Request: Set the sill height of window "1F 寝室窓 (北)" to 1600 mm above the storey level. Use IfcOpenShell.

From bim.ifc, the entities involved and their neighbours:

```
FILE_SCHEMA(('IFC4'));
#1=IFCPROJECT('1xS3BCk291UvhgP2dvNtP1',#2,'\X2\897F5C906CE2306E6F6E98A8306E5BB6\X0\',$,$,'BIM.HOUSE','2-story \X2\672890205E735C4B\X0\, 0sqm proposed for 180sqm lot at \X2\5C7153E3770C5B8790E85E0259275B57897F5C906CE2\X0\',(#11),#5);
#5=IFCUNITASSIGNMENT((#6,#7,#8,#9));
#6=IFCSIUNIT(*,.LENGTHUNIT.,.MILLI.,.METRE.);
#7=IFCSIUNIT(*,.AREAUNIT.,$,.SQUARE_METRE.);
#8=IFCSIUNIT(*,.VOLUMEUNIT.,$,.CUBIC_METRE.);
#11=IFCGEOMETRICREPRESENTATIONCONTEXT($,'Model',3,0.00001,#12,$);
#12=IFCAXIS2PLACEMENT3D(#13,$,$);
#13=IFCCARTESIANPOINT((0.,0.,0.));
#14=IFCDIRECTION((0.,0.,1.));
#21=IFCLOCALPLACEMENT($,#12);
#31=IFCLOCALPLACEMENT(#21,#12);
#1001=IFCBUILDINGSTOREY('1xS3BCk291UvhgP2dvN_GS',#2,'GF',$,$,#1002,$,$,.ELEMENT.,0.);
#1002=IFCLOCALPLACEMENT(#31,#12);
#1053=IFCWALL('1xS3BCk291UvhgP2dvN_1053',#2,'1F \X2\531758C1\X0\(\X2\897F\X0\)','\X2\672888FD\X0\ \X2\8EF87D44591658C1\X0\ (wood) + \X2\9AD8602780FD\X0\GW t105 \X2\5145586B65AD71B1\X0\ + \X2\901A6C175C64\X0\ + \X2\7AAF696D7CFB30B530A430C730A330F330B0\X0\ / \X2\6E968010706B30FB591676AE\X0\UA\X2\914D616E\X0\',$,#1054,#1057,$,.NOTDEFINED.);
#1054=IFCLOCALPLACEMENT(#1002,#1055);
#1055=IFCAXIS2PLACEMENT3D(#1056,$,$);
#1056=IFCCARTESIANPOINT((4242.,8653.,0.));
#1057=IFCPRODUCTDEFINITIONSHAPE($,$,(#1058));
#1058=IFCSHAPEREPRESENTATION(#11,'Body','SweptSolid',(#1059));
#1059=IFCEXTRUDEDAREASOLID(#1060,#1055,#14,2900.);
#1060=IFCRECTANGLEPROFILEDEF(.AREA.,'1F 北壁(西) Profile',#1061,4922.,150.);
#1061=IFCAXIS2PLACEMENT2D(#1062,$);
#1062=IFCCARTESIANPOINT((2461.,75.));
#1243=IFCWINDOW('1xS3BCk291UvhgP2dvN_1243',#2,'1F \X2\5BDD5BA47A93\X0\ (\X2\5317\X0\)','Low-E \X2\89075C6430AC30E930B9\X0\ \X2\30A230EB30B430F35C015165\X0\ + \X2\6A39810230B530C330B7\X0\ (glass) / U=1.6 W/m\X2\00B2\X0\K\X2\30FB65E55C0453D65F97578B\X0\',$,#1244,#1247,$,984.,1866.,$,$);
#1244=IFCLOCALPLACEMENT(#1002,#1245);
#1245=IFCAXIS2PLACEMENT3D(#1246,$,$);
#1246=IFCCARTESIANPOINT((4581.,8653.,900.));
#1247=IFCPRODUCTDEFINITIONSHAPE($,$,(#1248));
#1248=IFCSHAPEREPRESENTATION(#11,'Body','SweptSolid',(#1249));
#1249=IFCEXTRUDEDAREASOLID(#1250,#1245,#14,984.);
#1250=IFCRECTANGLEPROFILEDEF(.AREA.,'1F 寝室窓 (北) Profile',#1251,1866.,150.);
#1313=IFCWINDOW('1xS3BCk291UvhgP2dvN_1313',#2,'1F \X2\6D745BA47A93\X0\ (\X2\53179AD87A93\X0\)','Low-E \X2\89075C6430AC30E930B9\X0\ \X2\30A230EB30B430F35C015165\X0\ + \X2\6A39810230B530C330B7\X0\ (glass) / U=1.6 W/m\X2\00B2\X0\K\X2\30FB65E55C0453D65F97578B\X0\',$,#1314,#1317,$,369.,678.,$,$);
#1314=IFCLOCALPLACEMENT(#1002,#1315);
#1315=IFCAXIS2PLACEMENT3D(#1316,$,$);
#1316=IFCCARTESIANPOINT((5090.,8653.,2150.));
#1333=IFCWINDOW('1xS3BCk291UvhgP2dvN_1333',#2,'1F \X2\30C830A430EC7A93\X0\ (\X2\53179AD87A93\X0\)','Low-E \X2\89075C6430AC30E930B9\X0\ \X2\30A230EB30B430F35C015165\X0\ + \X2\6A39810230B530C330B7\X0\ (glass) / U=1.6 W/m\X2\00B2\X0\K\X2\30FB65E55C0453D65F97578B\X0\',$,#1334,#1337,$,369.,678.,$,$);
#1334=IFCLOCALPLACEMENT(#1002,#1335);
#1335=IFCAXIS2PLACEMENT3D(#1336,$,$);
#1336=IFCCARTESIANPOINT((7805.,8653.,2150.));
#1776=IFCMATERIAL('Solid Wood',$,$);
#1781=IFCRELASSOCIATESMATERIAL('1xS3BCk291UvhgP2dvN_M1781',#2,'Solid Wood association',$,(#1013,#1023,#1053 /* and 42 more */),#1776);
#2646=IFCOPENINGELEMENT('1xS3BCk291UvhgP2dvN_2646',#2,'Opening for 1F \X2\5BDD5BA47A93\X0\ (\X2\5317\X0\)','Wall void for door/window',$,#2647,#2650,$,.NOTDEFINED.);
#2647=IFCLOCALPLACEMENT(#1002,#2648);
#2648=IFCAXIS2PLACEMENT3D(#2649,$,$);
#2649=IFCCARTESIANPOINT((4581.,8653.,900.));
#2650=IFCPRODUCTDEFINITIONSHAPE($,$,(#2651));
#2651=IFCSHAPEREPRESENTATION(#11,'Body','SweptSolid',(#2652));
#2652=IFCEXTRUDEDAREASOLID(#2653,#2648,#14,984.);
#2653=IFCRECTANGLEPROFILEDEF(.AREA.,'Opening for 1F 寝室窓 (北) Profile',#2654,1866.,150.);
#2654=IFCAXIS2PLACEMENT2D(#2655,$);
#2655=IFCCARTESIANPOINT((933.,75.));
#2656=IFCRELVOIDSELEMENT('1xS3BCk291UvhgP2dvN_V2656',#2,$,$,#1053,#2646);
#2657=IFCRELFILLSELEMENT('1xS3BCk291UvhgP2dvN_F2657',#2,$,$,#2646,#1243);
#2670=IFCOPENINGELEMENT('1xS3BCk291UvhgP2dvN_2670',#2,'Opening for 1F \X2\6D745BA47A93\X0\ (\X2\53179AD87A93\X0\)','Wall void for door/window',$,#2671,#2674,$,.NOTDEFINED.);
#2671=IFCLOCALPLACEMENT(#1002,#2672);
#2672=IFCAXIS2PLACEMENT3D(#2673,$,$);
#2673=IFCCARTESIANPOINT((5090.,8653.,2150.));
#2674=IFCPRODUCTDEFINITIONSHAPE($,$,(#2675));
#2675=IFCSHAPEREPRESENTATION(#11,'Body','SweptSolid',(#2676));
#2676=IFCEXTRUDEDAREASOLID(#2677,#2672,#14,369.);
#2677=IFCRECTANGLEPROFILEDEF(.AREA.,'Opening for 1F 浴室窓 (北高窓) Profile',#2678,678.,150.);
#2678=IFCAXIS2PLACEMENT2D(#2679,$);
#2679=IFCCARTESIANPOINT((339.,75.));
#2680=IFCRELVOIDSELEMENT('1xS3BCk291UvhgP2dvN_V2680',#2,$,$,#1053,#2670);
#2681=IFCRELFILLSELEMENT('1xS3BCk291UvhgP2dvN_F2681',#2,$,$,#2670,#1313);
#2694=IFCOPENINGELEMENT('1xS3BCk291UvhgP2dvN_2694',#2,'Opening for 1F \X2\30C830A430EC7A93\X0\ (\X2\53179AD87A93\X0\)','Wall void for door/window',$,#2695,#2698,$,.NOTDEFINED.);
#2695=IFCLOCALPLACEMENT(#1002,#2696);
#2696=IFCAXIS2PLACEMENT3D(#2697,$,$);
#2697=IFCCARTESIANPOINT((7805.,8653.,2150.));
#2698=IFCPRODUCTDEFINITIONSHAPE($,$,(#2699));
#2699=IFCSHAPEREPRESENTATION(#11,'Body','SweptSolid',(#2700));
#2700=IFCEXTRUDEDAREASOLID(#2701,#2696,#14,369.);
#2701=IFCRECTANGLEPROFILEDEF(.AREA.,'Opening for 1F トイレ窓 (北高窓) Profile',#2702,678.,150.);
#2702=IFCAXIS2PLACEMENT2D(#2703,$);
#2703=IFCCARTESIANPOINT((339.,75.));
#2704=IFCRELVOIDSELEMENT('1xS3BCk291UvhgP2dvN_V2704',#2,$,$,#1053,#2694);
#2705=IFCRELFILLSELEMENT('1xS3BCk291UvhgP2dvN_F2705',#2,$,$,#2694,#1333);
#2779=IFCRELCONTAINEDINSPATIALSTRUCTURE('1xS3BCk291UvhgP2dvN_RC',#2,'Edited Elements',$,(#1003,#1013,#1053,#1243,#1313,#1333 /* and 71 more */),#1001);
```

```python
import numpy as np
import ifcopenshell
import ifcopenshell.api.geometry
import ifcopenshell.geom
import ifcopenshell.util.element
import ifcopenshell.util.placement
import ifcopenshell.util.shape
import ifcopenshell.util.unit

model = ifcopenshell.open("bim.ifc")
unit_scale = ifcopenshell.util.unit.calculate_unit_scale(model)

window = model.by_guid("1xS3BCk291UvhgP2dvN_1243")
opening = window.FillsVoids[0].RelatingOpeningElement
storey = ifcopenshell.util.element.get_container(window, ifc_class="IfcBuildingStorey")
level = ifcopenshell.util.placement.get_local_placement(storey.ObjectPlacement)[2, 3]

# The opening's origin need not be at the sill, so measure its lowest point.
shape = ifcopenshell.geom.create_shape(ifcopenshell.geom.settings(), opening)
bottom = ifcopenshell.util.shape.get_shape_bottom_elevation(shape, shape.geometry) / unit_scale
dz = level + 1600.0 - bottom

shift = np.array([0.0, 0.0, dz])
# The window is not placed relative to its opening, so move both.
for product in (opening, window):
    matrix = ifcopenshell.util.placement.get_local_placement(product.ObjectPlacement)
    matrix[:3, 3] += shift
    ifcopenshell.api.geometry.edit_object_placement(model, product=product, matrix=matrix, is_si=False)

print(f"moved by {dz * unit_scale:+.3f} m")

model.write("bim_v2.ifc")
```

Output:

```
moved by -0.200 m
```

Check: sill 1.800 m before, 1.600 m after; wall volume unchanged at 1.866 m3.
